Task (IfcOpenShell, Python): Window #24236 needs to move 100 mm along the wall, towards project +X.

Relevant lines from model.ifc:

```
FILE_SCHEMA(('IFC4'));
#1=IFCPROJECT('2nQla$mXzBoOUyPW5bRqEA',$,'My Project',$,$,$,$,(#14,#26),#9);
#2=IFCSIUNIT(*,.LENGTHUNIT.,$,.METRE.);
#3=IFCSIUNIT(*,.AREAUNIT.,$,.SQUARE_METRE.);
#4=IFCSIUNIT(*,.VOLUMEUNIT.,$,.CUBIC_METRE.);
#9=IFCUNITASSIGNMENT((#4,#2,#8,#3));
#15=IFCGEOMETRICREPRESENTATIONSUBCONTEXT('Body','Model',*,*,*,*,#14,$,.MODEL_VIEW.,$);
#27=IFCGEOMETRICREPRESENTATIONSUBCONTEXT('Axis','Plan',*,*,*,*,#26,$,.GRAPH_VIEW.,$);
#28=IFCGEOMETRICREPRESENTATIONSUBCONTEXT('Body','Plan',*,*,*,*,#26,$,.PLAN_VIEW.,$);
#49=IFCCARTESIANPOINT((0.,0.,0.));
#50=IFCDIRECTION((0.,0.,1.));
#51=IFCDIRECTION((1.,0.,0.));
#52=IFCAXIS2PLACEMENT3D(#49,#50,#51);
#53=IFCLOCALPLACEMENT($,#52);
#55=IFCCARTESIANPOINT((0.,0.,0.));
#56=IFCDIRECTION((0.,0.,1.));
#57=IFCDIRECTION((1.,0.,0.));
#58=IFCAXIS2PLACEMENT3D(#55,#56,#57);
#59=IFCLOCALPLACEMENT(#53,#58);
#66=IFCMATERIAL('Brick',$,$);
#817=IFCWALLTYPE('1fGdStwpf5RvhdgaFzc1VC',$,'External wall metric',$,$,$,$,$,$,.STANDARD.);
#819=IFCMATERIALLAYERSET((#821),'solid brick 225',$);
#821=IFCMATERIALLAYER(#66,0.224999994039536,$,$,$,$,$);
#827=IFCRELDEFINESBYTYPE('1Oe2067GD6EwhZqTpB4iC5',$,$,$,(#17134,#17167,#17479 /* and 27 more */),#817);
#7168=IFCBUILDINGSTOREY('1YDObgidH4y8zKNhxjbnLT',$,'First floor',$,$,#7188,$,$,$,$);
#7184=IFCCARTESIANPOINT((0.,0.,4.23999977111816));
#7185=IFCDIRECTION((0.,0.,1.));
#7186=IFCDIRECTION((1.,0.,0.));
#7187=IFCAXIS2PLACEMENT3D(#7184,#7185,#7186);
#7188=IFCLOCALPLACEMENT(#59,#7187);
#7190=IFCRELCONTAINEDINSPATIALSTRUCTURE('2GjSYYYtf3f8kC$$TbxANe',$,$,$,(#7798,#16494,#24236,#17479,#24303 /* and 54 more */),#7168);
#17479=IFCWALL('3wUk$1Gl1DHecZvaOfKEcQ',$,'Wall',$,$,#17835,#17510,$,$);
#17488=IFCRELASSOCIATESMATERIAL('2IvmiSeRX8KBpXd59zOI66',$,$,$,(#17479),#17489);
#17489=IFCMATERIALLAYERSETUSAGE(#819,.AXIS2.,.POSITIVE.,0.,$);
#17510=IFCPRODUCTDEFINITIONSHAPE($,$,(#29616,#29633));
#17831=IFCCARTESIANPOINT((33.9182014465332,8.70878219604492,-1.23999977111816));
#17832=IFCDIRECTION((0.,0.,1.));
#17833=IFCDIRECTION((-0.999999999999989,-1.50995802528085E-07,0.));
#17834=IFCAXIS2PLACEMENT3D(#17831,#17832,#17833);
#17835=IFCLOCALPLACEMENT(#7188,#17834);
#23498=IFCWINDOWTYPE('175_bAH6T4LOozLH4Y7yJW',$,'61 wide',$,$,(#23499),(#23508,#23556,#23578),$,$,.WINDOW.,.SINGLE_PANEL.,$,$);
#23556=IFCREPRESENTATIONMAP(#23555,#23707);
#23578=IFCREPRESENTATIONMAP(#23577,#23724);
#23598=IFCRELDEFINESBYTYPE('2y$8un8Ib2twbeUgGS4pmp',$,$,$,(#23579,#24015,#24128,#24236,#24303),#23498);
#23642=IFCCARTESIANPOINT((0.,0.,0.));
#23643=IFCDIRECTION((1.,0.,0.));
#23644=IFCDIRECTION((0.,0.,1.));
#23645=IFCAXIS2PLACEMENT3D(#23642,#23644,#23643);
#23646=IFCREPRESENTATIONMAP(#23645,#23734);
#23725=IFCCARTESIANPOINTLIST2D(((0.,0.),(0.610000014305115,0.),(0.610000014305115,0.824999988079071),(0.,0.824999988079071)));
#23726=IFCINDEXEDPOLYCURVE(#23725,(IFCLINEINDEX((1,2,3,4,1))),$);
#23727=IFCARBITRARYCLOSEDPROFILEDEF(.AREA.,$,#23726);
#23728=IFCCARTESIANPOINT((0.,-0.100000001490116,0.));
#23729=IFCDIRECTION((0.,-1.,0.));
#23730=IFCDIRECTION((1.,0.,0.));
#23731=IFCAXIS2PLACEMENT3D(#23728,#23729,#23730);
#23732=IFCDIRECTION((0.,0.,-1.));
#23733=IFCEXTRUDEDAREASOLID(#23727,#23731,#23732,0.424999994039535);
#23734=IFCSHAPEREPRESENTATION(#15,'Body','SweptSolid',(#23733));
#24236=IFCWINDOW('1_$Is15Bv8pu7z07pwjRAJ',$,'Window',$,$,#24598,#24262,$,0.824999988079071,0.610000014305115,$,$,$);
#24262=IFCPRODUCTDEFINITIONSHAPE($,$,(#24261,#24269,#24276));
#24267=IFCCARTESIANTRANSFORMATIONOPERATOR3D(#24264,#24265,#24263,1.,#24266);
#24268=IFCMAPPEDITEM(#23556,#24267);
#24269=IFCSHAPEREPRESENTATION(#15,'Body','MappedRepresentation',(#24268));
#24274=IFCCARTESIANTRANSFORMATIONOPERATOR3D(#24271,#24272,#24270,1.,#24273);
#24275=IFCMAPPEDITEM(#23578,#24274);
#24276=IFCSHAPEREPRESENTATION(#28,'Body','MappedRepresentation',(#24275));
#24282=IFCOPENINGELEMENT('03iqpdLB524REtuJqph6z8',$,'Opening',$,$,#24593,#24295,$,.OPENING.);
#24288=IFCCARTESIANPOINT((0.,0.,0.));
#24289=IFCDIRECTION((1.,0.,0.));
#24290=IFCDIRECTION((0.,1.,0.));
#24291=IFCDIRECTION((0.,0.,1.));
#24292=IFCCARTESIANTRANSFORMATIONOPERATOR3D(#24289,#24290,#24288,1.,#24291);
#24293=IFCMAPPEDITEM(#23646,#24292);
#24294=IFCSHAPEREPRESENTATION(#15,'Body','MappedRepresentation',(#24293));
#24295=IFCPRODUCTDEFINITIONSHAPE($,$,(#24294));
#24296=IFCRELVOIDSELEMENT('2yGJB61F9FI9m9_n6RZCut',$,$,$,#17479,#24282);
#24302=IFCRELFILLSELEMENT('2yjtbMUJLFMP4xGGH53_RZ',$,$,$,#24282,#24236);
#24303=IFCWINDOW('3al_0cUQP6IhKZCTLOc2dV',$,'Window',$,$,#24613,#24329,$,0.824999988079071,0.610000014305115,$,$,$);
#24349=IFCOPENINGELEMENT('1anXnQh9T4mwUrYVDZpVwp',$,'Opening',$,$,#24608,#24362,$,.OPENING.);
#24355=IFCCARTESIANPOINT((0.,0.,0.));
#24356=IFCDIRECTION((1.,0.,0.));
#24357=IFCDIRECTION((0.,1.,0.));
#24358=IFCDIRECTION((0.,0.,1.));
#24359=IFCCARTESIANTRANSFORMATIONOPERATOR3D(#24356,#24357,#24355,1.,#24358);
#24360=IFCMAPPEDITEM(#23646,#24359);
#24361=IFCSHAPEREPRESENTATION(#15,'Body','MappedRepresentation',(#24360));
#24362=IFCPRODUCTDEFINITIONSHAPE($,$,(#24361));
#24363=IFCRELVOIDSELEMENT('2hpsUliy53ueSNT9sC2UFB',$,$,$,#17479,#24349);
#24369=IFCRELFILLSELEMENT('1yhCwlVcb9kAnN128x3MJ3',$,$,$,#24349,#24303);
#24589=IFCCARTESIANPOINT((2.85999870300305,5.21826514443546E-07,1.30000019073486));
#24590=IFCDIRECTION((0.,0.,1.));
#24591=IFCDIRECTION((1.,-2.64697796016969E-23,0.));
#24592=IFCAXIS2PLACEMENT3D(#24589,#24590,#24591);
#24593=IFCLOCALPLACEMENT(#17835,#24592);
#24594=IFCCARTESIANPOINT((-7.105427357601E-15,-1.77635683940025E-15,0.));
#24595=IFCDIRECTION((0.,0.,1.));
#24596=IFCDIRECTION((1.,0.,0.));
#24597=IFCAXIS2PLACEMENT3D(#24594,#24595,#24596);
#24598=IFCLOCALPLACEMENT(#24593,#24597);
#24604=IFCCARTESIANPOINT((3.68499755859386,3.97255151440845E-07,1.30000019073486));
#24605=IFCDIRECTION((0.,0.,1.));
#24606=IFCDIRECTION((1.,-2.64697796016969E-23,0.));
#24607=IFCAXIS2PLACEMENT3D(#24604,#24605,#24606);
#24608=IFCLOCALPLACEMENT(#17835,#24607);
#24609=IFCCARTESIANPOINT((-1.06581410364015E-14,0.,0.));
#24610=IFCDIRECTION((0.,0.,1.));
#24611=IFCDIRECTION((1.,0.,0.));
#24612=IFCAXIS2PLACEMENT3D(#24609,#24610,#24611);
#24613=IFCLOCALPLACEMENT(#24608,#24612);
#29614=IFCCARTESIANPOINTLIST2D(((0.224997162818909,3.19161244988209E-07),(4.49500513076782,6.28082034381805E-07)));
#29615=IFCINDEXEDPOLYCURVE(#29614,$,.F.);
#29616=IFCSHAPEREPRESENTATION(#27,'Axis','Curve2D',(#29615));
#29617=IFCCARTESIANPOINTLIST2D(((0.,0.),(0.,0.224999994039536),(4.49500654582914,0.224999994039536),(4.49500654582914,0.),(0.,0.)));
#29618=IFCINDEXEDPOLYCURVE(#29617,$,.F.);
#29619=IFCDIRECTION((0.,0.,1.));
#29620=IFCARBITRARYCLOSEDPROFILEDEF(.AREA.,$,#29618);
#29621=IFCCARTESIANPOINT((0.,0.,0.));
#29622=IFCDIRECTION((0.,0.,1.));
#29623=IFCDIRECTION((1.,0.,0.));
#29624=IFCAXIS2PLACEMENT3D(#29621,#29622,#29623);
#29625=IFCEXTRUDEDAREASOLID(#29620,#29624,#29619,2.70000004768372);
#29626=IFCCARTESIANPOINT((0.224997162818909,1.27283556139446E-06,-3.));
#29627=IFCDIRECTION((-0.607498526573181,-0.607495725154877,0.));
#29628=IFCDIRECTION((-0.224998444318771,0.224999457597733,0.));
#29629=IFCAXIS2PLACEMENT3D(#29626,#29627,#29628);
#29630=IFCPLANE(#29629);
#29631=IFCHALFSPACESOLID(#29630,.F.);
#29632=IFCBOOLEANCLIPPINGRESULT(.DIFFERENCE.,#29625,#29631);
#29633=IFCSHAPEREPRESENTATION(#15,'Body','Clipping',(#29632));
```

```python
import ifcopenshell
import ifcopenshell.api.geometry
import ifcopenshell.util.placement
import ifcopenshell.util.unit

model = ifcopenshell.open("model.ifc")
unit_scale = ifcopenshell.util.unit.calculate_unit_scale(model)

window = model.by_id(24236)
opening = window.FillsVoids[0].RelatingOpeningElement
wall = opening.VoidsElements[0].RelatingBuildingElement

wall_matrix = ifcopenshell.util.placement.get_local_placement(wall.ObjectPlacement)
shift = wall_matrix[:3, 0] * -0.1 / unit_scale
before = ifcopenshell.util.placement.get_local_placement(window.ObjectPlacement)[:3, 3].copy()

# The window is placed relative to its opening, so it follows when the opening moves.
matrix = ifcopenshell.util.placement.get_local_placement(opening.ObjectPlacement)
matrix[:3, 3] += shift
ifcopenshell.api.geometry.edit_object_placement(
    model, product=opening, matrix=matrix, is_si=False, should_transform_children=True
)

after = ifcopenshell.util.placement.get_local_placement(window.ObjectPlacement)[:3, 3]
print("window moved by", (after - before).round(3) + 0.0)

model.write("model-out.ifc")
```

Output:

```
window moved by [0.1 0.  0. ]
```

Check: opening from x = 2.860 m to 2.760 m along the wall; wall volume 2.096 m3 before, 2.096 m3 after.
